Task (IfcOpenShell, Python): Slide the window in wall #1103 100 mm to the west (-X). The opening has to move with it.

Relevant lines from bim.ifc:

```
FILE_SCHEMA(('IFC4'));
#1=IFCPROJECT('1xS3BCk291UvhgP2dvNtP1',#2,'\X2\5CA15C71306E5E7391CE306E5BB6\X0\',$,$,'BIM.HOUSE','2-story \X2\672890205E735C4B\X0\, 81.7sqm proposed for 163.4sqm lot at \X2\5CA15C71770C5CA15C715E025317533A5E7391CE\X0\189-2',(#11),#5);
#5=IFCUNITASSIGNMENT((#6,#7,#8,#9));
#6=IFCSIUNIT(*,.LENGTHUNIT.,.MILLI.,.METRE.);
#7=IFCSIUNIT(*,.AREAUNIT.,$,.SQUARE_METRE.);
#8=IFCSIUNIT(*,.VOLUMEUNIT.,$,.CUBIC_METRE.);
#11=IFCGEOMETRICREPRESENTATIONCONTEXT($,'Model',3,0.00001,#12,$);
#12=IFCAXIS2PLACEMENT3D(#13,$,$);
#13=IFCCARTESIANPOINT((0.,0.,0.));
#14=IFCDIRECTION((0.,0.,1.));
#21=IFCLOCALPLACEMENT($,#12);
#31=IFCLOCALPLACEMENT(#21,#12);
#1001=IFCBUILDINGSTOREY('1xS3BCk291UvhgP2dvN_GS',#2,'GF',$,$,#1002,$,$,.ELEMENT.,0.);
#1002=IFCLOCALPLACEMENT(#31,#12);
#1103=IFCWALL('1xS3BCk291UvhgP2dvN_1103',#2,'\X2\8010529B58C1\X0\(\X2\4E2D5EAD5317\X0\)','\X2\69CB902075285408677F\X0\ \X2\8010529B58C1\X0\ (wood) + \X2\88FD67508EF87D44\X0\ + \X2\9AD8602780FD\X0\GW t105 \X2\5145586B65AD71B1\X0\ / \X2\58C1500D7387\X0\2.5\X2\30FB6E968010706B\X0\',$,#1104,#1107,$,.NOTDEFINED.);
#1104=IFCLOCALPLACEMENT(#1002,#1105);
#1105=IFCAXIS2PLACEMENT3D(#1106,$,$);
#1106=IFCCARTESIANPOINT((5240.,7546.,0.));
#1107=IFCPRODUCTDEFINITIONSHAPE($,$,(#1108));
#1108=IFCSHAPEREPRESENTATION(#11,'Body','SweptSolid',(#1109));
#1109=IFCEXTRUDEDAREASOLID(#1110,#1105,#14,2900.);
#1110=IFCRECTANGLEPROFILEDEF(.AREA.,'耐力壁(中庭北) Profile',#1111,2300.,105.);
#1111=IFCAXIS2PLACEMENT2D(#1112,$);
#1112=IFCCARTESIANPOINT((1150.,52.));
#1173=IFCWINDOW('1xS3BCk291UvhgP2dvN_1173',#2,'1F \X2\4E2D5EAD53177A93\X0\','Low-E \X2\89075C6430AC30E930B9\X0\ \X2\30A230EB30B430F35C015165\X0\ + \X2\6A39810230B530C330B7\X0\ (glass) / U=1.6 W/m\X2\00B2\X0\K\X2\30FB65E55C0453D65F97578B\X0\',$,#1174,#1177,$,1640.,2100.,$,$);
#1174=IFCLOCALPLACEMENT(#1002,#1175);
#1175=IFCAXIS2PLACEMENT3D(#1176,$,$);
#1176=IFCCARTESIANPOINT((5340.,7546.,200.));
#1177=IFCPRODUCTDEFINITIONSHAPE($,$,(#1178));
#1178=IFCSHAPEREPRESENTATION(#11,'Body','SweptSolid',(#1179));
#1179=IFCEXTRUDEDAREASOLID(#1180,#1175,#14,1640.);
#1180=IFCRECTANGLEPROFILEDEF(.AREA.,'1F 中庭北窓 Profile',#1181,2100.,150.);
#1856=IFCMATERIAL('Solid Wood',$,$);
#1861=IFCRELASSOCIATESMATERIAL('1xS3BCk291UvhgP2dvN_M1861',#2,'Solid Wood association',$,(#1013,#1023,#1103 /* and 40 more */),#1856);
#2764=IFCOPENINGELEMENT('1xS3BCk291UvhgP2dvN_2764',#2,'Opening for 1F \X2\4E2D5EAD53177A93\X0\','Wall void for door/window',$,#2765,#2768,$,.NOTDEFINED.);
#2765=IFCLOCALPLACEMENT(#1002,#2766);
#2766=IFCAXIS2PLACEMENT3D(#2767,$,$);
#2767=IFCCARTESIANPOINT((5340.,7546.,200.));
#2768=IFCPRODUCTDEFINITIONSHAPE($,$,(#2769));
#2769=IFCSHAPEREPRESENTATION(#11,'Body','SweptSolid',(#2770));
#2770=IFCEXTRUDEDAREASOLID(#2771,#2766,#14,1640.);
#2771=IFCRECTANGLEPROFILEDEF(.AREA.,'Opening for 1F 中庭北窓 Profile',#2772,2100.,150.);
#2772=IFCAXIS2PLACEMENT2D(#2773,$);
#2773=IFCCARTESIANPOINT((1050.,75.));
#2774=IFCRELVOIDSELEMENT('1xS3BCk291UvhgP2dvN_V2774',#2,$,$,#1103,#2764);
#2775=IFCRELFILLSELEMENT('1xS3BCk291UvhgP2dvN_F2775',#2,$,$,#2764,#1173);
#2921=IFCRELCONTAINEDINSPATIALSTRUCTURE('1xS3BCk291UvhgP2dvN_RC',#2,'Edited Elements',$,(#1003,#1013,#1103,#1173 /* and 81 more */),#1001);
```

```python
import ifcopenshell
import ifcopenshell.api.geometry
import ifcopenshell.util.placement
import ifcopenshell.util.unit

model = ifcopenshell.open("bim.ifc")
unit_scale = ifcopenshell.util.unit.calculate_unit_scale(model)

window = model.by_id(1173)
opening = window.FillsVoids[0].RelatingOpeningElement
wall = opening.VoidsElements[0].RelatingBuildingElement

wall_matrix = ifcopenshell.util.placement.get_local_placement(wall.ObjectPlacement)
shift = wall_matrix[:3, 0] * -0.1 / unit_scale
before = ifcopenshell.util.placement.get_local_placement(window.ObjectPlacement)[:3, 3].copy()

# The window is not placed relative to its opening, so move both.
for product in (opening, window):
    matrix = ifcopenshell.util.placement.get_local_placement(product.ObjectPlacement)
    matrix[:3, 3] += shift
    ifcopenshell.api.geometry.edit_object_placement(model, product=product, matrix=matrix, is_si=False)

after = ifcopenshell.util.placement.get_local_placement(window.ObjectPlacement)[:3, 3]
print("window moved by", (after - before).round(3) + 0.0)

model.write("bim-out.ifc")
```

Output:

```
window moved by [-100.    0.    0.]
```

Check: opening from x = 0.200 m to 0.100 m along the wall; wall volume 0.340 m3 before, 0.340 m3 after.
